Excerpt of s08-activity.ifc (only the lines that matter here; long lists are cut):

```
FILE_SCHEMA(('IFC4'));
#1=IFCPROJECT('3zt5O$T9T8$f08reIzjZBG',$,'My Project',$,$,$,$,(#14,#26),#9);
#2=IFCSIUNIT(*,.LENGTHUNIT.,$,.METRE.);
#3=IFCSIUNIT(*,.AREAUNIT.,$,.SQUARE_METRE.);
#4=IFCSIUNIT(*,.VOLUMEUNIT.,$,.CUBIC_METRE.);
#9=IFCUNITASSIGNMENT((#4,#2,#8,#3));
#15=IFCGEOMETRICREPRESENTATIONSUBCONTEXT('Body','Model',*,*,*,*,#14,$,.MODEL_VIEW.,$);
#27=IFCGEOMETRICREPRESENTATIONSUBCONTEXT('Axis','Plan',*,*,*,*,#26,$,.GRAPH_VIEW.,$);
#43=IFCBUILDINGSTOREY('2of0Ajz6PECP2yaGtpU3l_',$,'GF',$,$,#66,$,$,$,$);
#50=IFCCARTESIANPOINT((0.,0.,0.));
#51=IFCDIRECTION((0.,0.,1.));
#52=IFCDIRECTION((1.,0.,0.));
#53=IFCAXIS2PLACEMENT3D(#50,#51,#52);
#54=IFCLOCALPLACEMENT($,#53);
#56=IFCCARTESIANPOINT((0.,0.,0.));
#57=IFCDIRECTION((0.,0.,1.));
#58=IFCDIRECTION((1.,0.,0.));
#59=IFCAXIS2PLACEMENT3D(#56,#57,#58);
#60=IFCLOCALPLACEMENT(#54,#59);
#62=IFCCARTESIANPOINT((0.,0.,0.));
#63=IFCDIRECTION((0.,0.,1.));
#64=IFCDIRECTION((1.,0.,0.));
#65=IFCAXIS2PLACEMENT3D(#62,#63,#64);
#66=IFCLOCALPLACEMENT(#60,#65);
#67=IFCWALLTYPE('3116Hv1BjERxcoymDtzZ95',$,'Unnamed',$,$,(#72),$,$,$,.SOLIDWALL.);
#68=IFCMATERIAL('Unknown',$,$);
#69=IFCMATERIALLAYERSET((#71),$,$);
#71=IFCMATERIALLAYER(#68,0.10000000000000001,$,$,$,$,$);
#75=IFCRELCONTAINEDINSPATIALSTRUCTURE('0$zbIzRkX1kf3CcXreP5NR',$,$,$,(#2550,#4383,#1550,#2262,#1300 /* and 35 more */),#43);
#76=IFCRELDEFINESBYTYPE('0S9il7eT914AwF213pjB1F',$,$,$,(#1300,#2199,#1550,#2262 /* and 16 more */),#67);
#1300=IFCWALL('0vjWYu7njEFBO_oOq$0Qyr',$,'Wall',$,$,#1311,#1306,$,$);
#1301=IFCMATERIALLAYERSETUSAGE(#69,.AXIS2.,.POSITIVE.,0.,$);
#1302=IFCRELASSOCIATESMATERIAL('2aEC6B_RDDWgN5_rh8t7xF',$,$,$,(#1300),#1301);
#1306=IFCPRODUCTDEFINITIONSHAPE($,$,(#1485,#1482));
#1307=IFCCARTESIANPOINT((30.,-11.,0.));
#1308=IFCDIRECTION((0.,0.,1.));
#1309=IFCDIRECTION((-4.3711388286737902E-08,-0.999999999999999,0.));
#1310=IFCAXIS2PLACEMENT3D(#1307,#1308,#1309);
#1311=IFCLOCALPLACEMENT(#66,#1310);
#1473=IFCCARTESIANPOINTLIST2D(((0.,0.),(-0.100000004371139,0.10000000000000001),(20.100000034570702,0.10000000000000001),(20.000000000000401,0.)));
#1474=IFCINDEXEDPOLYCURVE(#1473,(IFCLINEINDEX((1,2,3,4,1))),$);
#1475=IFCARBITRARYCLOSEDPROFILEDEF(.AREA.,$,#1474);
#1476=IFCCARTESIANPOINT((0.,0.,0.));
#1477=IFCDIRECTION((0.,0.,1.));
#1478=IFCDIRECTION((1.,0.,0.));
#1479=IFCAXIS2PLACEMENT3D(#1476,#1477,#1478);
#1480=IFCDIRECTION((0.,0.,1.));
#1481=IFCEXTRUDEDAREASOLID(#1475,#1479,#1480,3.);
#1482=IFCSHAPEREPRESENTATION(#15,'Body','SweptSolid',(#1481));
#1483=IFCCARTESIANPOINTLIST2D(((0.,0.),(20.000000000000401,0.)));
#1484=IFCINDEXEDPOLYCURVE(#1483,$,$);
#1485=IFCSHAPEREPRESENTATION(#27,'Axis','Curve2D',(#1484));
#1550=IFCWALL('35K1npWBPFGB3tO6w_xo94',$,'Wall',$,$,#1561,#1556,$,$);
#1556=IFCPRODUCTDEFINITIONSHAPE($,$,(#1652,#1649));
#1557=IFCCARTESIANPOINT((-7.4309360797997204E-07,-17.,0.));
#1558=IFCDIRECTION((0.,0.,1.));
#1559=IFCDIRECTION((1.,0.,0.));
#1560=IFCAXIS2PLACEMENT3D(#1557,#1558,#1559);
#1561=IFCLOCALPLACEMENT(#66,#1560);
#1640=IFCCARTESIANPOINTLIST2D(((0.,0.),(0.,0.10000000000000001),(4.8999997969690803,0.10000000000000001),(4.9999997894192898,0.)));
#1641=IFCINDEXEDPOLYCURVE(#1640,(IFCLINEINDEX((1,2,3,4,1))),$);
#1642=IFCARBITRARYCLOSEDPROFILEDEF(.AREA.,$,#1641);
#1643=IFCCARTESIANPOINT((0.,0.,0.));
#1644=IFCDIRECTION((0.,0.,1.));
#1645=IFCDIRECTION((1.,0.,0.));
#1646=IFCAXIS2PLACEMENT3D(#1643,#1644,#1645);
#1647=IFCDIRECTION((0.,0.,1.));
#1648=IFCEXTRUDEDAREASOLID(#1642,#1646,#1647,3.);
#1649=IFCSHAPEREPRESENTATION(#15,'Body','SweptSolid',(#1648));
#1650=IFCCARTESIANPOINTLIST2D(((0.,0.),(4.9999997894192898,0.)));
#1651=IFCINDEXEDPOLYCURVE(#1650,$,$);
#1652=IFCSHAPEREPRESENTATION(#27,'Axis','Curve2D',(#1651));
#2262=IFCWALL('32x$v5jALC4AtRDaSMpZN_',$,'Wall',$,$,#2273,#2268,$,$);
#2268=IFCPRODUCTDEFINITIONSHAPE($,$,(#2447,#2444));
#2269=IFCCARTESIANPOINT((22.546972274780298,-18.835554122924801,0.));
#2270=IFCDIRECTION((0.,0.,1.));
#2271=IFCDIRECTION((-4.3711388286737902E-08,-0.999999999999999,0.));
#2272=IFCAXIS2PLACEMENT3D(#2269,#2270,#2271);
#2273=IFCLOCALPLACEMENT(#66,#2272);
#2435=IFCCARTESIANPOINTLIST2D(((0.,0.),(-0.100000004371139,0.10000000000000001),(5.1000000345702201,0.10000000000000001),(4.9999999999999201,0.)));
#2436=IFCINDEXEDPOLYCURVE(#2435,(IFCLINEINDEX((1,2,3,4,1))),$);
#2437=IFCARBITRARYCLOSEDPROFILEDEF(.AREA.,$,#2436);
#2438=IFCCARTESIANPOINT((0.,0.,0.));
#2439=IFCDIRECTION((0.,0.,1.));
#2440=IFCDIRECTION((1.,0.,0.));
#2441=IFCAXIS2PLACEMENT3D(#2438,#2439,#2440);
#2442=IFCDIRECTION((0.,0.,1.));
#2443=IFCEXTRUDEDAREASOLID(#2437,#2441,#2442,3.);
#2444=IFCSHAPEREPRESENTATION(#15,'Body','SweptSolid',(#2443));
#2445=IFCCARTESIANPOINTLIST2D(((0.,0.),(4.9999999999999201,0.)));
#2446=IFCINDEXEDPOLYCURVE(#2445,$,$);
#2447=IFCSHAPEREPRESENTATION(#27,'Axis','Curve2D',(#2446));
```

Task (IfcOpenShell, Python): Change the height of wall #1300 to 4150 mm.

```python
import ifcopenshell
import ifcopenshell.geom
import ifcopenshell.util.representation
import ifcopenshell.util.shape

model = ifcopenshell.open("s08-activity.ifc")
settings = ifcopenshell.geom.settings()


def volume(element):
    """Net volume in cubic metres, openings subtracted."""
    shape = ifcopenshell.geom.create_shape(settings, element)
    return ifcopenshell.util.shape.get_volume(shape.geometry)


wall = model.by_guid("0vjWYu7njEFBO_oOq$0Qyr")
before = volume(wall)

body = ifcopenshell.util.representation.get_representation(wall, "Model", "Body")
solid = body.Items[0]
old_height = solid.Depth
solid.Depth = 4.15
after = volume(wall)

print(f"height {old_height:g} -> {solid.Depth:g}, volume {before:.3f} -> {after:.3f} m3")

model.write("s08-activity-out.ifc")
```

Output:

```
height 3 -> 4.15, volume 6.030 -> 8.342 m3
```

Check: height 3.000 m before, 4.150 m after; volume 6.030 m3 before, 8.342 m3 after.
